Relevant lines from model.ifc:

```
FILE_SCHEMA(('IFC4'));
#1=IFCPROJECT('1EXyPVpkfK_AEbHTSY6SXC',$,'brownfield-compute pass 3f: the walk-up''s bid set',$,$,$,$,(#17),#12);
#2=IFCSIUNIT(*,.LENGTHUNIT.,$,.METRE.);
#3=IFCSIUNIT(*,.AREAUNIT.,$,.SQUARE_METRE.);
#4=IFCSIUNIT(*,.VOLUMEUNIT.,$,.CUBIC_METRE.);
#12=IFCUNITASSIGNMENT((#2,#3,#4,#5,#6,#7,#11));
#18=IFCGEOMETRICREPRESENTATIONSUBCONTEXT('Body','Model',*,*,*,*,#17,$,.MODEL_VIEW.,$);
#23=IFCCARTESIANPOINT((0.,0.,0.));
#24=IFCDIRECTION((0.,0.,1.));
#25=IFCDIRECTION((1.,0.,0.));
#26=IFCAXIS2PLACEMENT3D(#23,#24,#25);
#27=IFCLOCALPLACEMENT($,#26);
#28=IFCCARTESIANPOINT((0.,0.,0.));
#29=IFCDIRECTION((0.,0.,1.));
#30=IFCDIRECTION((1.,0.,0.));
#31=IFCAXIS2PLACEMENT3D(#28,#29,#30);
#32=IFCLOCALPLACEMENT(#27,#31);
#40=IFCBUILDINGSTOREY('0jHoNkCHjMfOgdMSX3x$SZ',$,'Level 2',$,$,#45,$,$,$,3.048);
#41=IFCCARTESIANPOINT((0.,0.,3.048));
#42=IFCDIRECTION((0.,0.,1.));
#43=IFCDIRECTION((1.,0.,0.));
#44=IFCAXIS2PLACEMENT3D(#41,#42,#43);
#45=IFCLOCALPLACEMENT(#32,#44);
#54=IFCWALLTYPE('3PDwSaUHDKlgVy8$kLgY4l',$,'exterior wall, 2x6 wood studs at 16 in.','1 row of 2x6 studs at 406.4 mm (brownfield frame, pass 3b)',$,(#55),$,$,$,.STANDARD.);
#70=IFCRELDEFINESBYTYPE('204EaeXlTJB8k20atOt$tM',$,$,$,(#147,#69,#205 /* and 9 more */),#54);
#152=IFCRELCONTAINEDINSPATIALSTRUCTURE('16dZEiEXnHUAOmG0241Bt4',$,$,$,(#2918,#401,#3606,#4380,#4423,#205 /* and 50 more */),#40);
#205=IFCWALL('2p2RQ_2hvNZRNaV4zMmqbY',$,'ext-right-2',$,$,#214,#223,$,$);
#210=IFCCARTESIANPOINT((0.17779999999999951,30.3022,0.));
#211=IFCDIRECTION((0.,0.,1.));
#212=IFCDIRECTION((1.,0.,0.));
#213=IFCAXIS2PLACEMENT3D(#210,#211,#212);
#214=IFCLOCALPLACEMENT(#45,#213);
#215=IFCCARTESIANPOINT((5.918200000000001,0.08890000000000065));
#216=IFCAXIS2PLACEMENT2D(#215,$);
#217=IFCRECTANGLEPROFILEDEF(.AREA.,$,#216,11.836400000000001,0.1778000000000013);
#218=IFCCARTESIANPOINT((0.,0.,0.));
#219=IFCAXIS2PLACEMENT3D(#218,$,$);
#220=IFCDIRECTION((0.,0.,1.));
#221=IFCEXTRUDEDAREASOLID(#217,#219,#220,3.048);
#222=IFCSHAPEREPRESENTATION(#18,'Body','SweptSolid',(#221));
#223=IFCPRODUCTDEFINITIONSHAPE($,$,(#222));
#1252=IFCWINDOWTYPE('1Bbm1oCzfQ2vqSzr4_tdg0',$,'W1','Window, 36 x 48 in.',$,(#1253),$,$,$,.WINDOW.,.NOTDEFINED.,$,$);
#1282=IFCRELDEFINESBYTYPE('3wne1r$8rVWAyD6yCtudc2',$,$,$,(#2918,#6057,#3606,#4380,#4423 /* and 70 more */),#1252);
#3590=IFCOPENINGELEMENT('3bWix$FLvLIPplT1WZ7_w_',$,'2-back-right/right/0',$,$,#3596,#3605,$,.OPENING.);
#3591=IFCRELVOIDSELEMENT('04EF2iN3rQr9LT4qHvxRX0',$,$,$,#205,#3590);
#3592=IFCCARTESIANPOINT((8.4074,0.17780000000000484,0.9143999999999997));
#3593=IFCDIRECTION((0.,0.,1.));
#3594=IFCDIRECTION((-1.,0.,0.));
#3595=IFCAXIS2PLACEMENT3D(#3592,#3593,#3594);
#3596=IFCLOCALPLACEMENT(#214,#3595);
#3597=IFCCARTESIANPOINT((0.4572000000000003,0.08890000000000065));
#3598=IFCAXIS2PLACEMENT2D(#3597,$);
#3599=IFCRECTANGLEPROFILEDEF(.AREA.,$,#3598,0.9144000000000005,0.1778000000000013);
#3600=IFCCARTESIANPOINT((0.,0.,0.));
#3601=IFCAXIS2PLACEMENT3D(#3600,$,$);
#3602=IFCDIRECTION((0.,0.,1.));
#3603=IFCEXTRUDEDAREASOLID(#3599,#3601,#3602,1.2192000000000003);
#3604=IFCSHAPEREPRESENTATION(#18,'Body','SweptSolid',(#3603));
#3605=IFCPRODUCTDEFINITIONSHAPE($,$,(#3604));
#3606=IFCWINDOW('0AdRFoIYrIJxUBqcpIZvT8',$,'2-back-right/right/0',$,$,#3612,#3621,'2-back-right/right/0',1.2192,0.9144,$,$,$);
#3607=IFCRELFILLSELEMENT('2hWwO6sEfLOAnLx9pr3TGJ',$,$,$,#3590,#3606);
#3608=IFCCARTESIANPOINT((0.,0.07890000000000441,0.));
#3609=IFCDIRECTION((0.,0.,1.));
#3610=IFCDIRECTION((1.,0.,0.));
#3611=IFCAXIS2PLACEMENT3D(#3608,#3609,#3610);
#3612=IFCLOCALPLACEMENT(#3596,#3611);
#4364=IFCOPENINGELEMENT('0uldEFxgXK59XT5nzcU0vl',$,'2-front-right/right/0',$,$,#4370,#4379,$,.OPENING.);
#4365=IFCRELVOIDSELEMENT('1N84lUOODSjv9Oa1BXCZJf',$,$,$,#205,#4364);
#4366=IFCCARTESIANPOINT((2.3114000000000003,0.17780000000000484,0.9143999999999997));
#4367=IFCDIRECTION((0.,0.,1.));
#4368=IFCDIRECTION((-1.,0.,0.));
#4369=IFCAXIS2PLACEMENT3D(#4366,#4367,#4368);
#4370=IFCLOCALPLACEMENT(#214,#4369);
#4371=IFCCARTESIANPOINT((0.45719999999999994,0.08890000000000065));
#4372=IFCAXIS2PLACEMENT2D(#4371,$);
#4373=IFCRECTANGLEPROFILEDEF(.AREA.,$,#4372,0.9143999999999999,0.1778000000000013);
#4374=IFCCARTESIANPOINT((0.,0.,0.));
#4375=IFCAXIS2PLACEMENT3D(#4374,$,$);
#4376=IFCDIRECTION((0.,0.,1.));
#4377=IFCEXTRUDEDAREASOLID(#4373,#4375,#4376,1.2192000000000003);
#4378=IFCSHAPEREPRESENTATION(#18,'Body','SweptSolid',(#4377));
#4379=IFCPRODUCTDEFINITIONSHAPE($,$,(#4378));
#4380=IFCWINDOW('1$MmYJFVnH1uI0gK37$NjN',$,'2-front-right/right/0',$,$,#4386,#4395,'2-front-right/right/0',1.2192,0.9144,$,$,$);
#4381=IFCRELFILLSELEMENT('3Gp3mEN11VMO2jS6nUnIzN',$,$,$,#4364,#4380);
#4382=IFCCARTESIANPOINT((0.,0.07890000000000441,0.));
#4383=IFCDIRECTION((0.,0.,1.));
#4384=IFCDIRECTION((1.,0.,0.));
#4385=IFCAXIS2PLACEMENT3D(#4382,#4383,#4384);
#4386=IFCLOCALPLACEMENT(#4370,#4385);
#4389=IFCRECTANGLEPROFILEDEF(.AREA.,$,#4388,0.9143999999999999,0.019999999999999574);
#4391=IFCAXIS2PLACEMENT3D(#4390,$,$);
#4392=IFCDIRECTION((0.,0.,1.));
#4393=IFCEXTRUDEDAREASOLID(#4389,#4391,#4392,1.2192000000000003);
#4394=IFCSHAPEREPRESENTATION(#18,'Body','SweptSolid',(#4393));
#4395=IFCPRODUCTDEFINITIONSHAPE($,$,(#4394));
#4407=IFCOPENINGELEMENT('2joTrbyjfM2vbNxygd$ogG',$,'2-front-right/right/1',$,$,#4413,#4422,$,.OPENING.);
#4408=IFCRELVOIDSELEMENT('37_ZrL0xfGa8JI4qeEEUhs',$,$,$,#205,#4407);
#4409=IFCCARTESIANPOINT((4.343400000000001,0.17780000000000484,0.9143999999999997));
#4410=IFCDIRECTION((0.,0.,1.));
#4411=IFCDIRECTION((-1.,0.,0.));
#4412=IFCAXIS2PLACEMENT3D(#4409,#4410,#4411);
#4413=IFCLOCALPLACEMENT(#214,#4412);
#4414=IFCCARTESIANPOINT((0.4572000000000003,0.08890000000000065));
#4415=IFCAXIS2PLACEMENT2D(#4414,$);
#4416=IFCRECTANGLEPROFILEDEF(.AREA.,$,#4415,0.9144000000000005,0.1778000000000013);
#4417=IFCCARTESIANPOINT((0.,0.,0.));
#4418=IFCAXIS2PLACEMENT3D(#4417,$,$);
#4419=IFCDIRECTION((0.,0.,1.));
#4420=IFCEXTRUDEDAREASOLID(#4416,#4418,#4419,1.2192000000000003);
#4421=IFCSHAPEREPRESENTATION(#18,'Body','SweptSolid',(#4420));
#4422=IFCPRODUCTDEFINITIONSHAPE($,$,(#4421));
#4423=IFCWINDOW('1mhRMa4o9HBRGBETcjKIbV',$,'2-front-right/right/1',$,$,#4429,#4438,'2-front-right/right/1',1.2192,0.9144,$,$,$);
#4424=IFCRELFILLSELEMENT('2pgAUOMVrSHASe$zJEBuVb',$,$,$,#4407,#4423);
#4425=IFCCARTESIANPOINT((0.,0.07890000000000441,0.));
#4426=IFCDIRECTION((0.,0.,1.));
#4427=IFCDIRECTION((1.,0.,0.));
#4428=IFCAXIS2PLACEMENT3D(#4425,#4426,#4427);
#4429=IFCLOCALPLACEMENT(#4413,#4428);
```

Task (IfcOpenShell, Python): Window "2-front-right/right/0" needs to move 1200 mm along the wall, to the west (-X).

```python
import ifcopenshell
import ifcopenshell.api.geometry
import ifcopenshell.util.placement
import ifcopenshell.util.unit

model = ifcopenshell.open("model.ifc")
unit_scale = ifcopenshell.util.unit.calculate_unit_scale(model)

window = model.by_guid("1$MmYJFVnH1uI0gK37$NjN")
opening = window.FillsVoids[0].RelatingOpeningElement
wall = opening.VoidsElements[0].RelatingBuildingElement

wall_matrix = ifcopenshell.util.placement.get_local_placement(wall.ObjectPlacement)
shift = wall_matrix[:3, 0] * -1.2 / unit_scale
before = ifcopenshell.util.placement.get_local_placement(window.ObjectPlacement)[:3, 3].copy()

# The window is placed relative to its opening, so it follows when the opening moves.
matrix = ifcopenshell.util.placement.get_local_placement(opening.ObjectPlacement)
matrix[:3, 3] += shift
ifcopenshell.api.geometry.edit_object_placement(
    model, product=opening, matrix=matrix, is_si=False, should_transform_children=True
)

after = ifcopenshell.util.placement.get_local_placement(window.ObjectPlacement)[:3, 3]
print("window moved by", (after - before).round(3) + 0.0)

model.write("model_updated.ifc")
```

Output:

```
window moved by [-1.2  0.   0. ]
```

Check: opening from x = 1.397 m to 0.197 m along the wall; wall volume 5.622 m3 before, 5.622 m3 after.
